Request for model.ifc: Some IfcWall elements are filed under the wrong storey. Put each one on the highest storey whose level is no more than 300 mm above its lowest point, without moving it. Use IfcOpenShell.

First a look at what the model holds.

```python
import ifcopenshell
import ifcopenshell.util.element
import ifcopenshell.util.placement

model = ifcopenshell.open("model.ifc")
print(model.schema)
for storey in model.by_type("IfcBuildingStorey"):
    level = ifcopenshell.util.placement.get_storey_elevation(storey)
    count = sum(e.is_a("IfcWall") for e in ifcopenshell.util.element.get_contained(storey))
    print(storey.id(), storey.Name, round(level, 3), count, sep=" | ")
```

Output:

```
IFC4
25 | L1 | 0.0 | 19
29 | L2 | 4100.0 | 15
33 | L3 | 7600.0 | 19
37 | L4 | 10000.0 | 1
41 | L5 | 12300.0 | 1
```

```python
import ifcopenshell
import ifcopenshell.api.spatial
import ifcopenshell.geom
import ifcopenshell.util.element
import ifcopenshell.util.placement
import ifcopenshell.util.shape
import ifcopenshell.util.unit

model = ifcopenshell.open("model.ifc")
unit_scale = ifcopenshell.util.unit.calculate_unit_scale(model)
settings = ifcopenshell.geom.settings()

levels = sorted(
    ((ifcopenshell.util.placement.get_storey_elevation(s) * unit_scale, s) for s in model.by_type("IfcBuildingStorey")),
    key=lambda pair: pair[0],
)

for e in model.by_type("IfcWall"):
    current = e.ContainedInStructure[0].RelatingStructure if e.ContainedInStructure else None
    if current is None or not current.is_a("IfcBuildingStorey"):
        continue
    shape = ifcopenshell.geom.create_shape(settings, e)
    bottom = ifcopenshell.util.shape.get_shape_bottom_elevation(shape, shape.geometry)
    below = [s for level, s in levels if level <= bottom + 0.3]
    storey = below[-1] if below else levels[0][1]
    if storey != current:
        # assign_container keeps the world position.
        ifcopenshell.api.spatial.assign_container(model, products=[e], relating_structure=storey)
        print(e.id(), current.Name, "->", storey.Name)

model.write("model_v2.ifc")
```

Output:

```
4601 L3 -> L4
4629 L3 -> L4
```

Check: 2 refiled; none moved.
